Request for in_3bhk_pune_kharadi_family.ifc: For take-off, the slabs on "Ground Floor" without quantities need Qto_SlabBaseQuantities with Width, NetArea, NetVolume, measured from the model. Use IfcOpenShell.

First a look at what the model holds.

```python
import ifcopenshell
import ifcopenshell.util.element
import ifcopenshell.util.unit

model = ifcopenshell.open("in_3bhk_pune_kharadi_family.ifc")
print(model.schema)
for unit_type in ("LENGTHUNIT", "AREAUNIT", "VOLUMEUNIT"):
    print(unit_type, ifcopenshell.util.unit.calculate_unit_scale(model, unit_type))
storey = next(s for s in model.by_type("IfcBuildingStorey") if s.Name == "Ground Floor")
slabs = [e for e in ifcopenshell.util.element.get_decomposition(storey) if e.is_a("IfcSlab")]
for e in sorted(slabs, key=lambda e: e.id()):
    print(e.id(), e.is_a(), e.Name, list(ifcopenshell.util.element.get_psets(e, qtos_only=True)), sep=" | ")
```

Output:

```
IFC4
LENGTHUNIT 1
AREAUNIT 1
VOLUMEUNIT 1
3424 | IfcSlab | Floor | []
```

```python
import ifcopenshell
import ifcopenshell.api.pset
import ifcopenshell.geom
import ifcopenshell.util.element
import ifcopenshell.util.shape
import ifcopenshell.util.unit

model = ifcopenshell.open("in_3bhk_pune_kharadi_family.ifc")
unit_scale = ifcopenshell.util.unit.calculate_unit_scale(model)
area_scale = ifcopenshell.util.unit.calculate_unit_scale(model, "AREAUNIT")
volume_scale = ifcopenshell.util.unit.calculate_unit_scale(model, "VOLUMEUNIT")
settings = ifcopenshell.geom.settings()

storey = next(s for s in model.by_type("IfcBuildingStorey") if s.Name == "Ground Floor")
slabs = [e for e in ifcopenshell.util.element.get_decomposition(storey) if e.is_a("IfcSlab")]

for e in sorted(slabs, key=lambda e: e.id()):
    if ifcopenshell.util.element.get_psets(e, qtos_only=True, should_inherit=False):
        continue
    # Geometry comes back in metres, in the element's own axes.
    shape = ifcopenshell.geom.create_shape(settings, e)
    values = {
        "Width": ifcopenshell.util.shape.get_z(shape.geometry) / unit_scale,
        "NetArea": ifcopenshell.util.shape.get_footprint_area(shape.geometry) / area_scale,
        "NetVolume": ifcopenshell.util.shape.get_volume(shape.geometry) / volume_scale,
    }
    qto = ifcopenshell.api.pset.add_qto(model, product=e, name="Qto_SlabBaseQuantities")
    ifcopenshell.api.pset.edit_qto(model, qto=qto, properties=values)
    print(e.id(), {k: round(v, 3) for k, v in values.items()})

model.write("in_3bhk_pune_kharadi_family_edited.ifc")
```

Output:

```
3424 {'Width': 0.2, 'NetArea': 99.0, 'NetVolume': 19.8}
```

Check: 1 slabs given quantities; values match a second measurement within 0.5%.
